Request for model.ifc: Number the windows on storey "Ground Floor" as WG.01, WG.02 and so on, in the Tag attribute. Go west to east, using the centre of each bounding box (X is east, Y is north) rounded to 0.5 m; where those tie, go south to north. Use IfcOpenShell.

First a look at what the model holds.

```python
import ifcopenshell
import ifcopenshell.util.element
import ifcopenshell.util.placement

model = ifcopenshell.open("model.ifc")
print(model.schema)
storey = next(s for s in model.by_type("IfcBuildingStorey") if s.Name == "Ground Floor")
windows = [e for e in ifcopenshell.util.element.get_decomposition(storey) if e.is_a("IfcWindow")]
for e in sorted(windows, key=lambda e: e.id()):
    origin = ifcopenshell.util.placement.get_local_placement(e.ObjectPlacement)[:3, 3]
    print(e.id(), e.Tag, e.Name, origin.round(2) + 0.0, sep=" | ")
```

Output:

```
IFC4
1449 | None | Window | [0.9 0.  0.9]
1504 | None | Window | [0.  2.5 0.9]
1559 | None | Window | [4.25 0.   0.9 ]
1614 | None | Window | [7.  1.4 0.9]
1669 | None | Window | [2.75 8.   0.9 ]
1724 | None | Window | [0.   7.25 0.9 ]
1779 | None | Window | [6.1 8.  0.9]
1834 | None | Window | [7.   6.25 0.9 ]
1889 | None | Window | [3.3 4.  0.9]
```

```python
import ifcopenshell
import ifcopenshell.geom
import ifcopenshell.util.element
import ifcopenshell.util.shape

model = ifcopenshell.open("model.ifc")
settings = ifcopenshell.geom.settings()
settings.set("use-world-coords", True)


def centre(element):
    shape = ifcopenshell.geom.create_shape(settings, element)
    return ifcopenshell.util.shape.get_bbox_centroid(shape.geometry)


storey = next(s for s in model.by_type("IfcBuildingStorey") if s.Name == "Ground Floor")
windows = [e for e in ifcopenshell.util.element.get_decomposition(storey) if e.is_a("IfcWindow")]

# Insertion points can sit at a corner or the storey origin, so sort by the geometry (in metres).
centres = {e: centre(e) for e in windows}
windows.sort(key=lambda e: (round(centres[e][0] / 0.5), centres[e][1]))

for i, e in enumerate(windows, start=1):
    number = f"WG.{i:02d}"
    e.Tag = number
    print(e.id(), number)

model.write("model_v2.ifc")
```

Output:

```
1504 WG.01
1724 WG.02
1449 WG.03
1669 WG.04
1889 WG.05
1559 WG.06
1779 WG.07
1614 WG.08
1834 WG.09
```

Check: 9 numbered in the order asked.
